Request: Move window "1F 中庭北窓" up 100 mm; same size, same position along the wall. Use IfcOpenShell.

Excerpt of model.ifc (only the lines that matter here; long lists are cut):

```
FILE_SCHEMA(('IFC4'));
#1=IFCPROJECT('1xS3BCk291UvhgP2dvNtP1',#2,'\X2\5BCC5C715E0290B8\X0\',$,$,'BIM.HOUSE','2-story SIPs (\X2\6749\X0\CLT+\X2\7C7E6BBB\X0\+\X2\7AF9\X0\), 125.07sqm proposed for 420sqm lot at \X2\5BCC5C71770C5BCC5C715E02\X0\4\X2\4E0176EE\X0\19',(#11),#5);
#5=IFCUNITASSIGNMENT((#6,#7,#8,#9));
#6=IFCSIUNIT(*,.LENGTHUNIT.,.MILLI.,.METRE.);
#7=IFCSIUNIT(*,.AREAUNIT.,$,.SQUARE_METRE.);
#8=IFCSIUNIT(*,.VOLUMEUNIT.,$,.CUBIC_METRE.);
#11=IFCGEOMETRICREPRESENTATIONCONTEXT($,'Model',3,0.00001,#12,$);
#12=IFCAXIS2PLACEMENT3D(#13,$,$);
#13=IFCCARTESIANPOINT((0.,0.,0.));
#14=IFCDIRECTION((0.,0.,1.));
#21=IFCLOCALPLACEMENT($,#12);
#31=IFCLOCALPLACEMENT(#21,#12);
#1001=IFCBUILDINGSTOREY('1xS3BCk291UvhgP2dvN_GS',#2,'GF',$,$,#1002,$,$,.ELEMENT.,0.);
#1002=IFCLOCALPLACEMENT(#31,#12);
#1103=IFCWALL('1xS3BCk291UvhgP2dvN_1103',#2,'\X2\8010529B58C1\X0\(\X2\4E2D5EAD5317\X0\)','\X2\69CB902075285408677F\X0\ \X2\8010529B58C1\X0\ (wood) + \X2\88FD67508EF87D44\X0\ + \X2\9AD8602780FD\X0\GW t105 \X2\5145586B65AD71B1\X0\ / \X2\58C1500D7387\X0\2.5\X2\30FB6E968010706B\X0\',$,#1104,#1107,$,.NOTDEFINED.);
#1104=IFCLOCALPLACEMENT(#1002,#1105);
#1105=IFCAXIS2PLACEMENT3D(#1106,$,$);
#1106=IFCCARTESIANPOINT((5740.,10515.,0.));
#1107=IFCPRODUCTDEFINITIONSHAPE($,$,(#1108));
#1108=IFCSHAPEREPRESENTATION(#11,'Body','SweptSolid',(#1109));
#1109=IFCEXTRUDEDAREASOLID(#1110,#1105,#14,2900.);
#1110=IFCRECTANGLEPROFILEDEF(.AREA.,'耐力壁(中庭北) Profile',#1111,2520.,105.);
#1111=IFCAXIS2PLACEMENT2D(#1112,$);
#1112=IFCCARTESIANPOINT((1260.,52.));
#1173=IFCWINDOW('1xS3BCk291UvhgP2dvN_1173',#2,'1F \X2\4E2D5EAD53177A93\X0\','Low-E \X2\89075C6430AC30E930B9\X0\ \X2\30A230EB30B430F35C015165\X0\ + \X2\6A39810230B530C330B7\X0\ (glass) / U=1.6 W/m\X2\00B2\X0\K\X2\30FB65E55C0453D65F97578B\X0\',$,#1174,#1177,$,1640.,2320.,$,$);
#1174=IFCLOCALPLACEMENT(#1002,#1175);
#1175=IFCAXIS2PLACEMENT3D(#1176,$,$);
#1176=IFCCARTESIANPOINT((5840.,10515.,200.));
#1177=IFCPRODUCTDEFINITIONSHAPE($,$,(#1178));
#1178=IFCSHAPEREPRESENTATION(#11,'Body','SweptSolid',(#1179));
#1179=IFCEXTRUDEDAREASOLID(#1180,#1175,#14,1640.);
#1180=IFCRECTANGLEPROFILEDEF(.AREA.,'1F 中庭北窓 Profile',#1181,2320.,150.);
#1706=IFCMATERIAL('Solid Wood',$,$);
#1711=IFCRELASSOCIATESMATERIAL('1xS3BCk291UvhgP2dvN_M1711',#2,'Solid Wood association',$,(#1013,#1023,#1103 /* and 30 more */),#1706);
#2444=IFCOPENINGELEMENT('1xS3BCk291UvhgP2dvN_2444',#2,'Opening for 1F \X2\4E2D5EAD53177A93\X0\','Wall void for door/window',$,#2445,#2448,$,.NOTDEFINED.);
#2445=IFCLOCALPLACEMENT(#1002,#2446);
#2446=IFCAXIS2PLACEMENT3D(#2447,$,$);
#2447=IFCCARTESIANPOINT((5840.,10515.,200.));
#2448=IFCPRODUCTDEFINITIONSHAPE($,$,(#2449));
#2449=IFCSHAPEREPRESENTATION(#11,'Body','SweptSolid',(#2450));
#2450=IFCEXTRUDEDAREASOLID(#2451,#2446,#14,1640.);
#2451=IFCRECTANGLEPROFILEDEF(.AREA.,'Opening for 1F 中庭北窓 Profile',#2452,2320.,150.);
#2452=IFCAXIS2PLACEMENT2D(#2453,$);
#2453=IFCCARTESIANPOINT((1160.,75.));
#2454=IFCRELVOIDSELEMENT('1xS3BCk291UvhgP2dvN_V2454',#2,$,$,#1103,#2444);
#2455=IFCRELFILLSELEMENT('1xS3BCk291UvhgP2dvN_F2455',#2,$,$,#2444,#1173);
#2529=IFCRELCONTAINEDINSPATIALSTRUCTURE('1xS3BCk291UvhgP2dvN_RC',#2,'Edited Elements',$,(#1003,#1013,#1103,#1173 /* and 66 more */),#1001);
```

```python
import numpy as np
import ifcopenshell
import ifcopenshell.api.geometry
import ifcopenshell.util.placement
import ifcopenshell.util.unit

model = ifcopenshell.open("model.ifc")
unit_scale = ifcopenshell.util.unit.calculate_unit_scale(model)

window = model.by_id(1173)
opening = window.FillsVoids[0].RelatingOpeningElement
dz = 0.1 / unit_scale

shift = np.array([0.0, 0.0, dz])
# The window is not placed relative to its opening, so move both.
for product in (opening, window):
    matrix = ifcopenshell.util.placement.get_local_placement(product.ObjectPlacement)
    matrix[:3, 3] += shift
    ifcopenshell.api.geometry.edit_object_placement(model, product=product, matrix=matrix, is_si=False)

print(f"moved by {dz * unit_scale:+.3f} m")

model.write("model_v2.ifc")
```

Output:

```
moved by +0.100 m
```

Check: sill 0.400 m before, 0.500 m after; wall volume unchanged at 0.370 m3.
